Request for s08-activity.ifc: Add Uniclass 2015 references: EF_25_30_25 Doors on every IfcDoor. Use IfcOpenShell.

First a look at what the model holds.

```python
import ifcopenshell

model = ifcopenshell.open("s08-activity.ifc")
print(model.schema)
print("classifications:", [c.Name for c in model.by_type("IfcClassification")])
for ifc_class in ("IfcDoor", "IfcRoof", "IfcStair", "IfcWall", "IfcWindow"):
    print(ifc_class, len(model.by_type(ifc_class)))
```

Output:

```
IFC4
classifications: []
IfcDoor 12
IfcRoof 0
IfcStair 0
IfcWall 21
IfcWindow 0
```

```python
import ifcopenshell
import ifcopenshell.api.classification

model = ifcopenshell.open("s08-activity.ifc")

system = ifcopenshell.api.classification.add_classification(model, classification="Uniclass 2015")

codes = {
    "IfcDoor": ("EF_25_30_25", "Doors"),
}
for ifc_class, (code, name) in codes.items():
    products = model.by_type(ifc_class)
    ifcopenshell.api.classification.add_reference(
        model, products=products, classification=system, identification=code, name=name
    )
    print(code, len(products))

model.write("s08-activity_edited.ifc")
```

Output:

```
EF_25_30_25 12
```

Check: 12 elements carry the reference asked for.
